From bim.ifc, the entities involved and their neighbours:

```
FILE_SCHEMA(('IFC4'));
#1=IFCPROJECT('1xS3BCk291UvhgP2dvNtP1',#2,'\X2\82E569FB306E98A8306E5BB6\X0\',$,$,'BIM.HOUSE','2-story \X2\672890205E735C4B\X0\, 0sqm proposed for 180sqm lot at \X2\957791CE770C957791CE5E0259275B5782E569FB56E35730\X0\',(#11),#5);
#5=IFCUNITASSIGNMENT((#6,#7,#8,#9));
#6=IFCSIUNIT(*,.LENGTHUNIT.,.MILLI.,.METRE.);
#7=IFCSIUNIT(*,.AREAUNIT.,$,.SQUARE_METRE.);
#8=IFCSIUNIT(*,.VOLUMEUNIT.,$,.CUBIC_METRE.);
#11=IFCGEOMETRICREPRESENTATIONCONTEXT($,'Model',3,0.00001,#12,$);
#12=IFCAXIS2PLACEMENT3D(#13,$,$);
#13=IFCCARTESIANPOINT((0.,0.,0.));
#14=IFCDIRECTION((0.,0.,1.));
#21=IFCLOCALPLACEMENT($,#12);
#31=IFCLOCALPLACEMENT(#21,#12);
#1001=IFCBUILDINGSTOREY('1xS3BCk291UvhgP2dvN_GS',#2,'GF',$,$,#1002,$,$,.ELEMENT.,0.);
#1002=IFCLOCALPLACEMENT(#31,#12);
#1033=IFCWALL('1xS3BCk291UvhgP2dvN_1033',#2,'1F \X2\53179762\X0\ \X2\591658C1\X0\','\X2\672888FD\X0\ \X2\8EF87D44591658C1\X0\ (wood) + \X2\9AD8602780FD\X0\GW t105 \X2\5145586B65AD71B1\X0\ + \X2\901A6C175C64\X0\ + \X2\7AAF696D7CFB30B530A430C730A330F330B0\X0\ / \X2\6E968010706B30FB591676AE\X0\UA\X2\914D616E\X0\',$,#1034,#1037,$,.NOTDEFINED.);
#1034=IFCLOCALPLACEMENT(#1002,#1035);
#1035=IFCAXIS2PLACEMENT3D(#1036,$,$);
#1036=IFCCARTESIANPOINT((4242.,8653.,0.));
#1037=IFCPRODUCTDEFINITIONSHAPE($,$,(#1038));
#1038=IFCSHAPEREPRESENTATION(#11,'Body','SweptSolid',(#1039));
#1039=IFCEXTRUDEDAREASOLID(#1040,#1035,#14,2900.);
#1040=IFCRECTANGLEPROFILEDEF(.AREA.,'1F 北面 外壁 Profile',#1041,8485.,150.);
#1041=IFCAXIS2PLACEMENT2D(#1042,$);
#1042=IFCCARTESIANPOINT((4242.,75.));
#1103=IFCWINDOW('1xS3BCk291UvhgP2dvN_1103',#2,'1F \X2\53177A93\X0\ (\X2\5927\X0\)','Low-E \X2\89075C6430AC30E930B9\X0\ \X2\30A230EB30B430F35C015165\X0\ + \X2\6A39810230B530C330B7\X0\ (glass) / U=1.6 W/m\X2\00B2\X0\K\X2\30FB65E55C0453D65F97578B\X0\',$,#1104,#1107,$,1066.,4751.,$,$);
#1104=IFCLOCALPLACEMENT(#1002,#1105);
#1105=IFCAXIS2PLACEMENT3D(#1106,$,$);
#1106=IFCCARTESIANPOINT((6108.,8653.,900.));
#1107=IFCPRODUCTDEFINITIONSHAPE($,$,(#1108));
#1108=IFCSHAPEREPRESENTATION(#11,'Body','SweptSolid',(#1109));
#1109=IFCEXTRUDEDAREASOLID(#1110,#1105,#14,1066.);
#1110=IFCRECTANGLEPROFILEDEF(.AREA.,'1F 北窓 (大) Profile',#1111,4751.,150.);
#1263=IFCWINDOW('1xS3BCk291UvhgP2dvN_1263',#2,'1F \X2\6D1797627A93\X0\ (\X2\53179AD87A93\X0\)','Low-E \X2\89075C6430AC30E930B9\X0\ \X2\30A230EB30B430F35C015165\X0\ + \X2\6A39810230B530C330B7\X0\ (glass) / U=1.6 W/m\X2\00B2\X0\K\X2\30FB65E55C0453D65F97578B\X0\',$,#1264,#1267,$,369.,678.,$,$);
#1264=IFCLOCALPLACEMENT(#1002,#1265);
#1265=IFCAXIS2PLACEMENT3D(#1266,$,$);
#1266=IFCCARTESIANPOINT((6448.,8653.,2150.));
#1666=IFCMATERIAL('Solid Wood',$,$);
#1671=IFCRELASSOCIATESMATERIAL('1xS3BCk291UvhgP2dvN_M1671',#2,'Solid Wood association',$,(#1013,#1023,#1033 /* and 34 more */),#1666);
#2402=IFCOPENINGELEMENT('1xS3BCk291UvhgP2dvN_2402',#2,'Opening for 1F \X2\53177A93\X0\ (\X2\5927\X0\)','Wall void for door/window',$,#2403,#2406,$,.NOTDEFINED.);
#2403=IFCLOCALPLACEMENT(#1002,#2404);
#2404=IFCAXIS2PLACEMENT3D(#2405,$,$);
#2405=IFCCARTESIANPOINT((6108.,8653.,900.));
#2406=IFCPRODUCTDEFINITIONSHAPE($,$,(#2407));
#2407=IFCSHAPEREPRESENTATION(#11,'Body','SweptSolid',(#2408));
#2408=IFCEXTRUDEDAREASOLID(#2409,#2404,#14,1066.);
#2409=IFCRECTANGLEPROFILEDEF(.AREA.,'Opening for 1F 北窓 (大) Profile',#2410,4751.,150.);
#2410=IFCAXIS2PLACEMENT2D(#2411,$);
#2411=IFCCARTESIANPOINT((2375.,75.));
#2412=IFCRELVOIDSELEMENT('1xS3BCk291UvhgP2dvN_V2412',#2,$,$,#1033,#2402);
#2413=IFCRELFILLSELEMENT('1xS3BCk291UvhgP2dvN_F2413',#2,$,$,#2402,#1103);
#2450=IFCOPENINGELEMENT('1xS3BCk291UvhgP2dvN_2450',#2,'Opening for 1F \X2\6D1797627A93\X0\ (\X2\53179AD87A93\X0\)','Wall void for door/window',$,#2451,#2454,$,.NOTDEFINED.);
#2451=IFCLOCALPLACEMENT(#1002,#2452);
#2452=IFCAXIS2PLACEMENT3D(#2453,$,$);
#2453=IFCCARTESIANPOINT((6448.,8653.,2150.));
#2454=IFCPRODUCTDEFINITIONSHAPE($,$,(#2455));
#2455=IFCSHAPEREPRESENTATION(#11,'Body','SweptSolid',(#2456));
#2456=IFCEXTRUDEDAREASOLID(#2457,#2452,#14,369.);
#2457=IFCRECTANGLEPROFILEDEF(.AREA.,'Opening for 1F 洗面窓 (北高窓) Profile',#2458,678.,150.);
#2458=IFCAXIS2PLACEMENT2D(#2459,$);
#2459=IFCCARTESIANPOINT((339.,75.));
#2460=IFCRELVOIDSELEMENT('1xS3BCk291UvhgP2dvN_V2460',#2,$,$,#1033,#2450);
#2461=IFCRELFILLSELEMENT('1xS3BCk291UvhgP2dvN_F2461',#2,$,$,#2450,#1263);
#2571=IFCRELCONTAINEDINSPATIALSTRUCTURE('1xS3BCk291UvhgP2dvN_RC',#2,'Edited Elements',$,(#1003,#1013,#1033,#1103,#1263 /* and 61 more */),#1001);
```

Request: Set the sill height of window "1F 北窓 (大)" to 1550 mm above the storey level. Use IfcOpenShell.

```python
import numpy as np
import ifcopenshell
import ifcopenshell.api.geometry
import ifcopenshell.geom
import ifcopenshell.util.element
import ifcopenshell.util.placement
import ifcopenshell.util.shape
import ifcopenshell.util.unit

model = ifcopenshell.open("bim.ifc")
unit_scale = ifcopenshell.util.unit.calculate_unit_scale(model)

window = model.by_guid("1xS3BCk291UvhgP2dvN_1103")
opening = window.FillsVoids[0].RelatingOpeningElement
storey = ifcopenshell.util.element.get_container(window, ifc_class="IfcBuildingStorey")
level = ifcopenshell.util.placement.get_local_placement(storey.ObjectPlacement)[2, 3]

# The opening's origin need not be at the sill, so measure its lowest point.
shape = ifcopenshell.geom.create_shape(ifcopenshell.geom.settings(), opening)
bottom = ifcopenshell.util.shape.get_shape_bottom_elevation(shape, shape.geometry) / unit_scale
dz = level + 1550.0 - bottom

shift = np.array([0.0, 0.0, dz])
# The window is not placed relative to its opening, so move both.
for product in (opening, window):
    matrix = ifcopenshell.util.placement.get_local_placement(product.ObjectPlacement)
    matrix[:3, 3] += shift
    ifcopenshell.api.geometry.edit_object_placement(model, product=product, matrix=matrix, is_si=False)

print(f"moved by {dz * unit_scale:+.3f} m")

model.write("bim_v2.ifc")
```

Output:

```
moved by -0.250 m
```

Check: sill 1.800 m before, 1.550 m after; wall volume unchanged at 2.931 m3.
